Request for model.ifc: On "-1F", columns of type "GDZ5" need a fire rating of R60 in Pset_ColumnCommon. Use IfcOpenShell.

First a look at what the model holds.

```python
import ifcopenshell
import ifcopenshell.util.element

model = ifcopenshell.open("model.ifc")
print(model.schema)
storey = next(s for s in model.by_type("IfcBuildingStorey") if s.Name == "-1F")
columns = [e for e in ifcopenshell.util.element.get_decomposition(storey) if e.is_a("IfcColumn")]
seen = {}
for e in columns:
    element_type = ifcopenshell.util.element.get_type(e)
    key = (element_type.Name if element_type != e and element_type else None, ifcopenshell.util.element.get_pset(e, "Pset_ColumnCommon", "FireRating"))
    seen[key] = seen.get(key, 0) + 1
for (name, value), count in sorted(seen.items(), key=str):
    print(count, "x", name, "|", value)
```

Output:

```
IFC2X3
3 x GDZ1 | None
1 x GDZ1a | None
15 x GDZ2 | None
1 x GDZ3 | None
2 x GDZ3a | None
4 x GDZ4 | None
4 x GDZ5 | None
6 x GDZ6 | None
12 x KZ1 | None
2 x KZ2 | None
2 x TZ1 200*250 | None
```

```python
import ifcopenshell
import ifcopenshell.api.pset
import ifcopenshell.util.element

model = ifcopenshell.open("model.ifc")

storey = next(s for s in model.by_type("IfcBuildingStorey") if s.Name == "-1F")
columns = [e for e in ifcopenshell.util.element.get_decomposition(storey) if e.is_a("IfcColumn")]

count = 0
for e in columns:
    element_type = ifcopenshell.util.element.get_type(e)
    if element_type in (None, e) or element_type.Name != "GDZ5":
        continue
    # add_pset returns the element's existing set when there is one.
    pset = ifcopenshell.api.pset.add_pset(model, product=e, name="Pset_ColumnCommon")
    ifcopenshell.api.pset.edit_pset(model, pset=pset, properties={"FireRating": "R60"})
    count += 1

print(count, "columns updated")

model.write("model_v2.ifc")
```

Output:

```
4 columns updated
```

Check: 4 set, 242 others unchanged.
